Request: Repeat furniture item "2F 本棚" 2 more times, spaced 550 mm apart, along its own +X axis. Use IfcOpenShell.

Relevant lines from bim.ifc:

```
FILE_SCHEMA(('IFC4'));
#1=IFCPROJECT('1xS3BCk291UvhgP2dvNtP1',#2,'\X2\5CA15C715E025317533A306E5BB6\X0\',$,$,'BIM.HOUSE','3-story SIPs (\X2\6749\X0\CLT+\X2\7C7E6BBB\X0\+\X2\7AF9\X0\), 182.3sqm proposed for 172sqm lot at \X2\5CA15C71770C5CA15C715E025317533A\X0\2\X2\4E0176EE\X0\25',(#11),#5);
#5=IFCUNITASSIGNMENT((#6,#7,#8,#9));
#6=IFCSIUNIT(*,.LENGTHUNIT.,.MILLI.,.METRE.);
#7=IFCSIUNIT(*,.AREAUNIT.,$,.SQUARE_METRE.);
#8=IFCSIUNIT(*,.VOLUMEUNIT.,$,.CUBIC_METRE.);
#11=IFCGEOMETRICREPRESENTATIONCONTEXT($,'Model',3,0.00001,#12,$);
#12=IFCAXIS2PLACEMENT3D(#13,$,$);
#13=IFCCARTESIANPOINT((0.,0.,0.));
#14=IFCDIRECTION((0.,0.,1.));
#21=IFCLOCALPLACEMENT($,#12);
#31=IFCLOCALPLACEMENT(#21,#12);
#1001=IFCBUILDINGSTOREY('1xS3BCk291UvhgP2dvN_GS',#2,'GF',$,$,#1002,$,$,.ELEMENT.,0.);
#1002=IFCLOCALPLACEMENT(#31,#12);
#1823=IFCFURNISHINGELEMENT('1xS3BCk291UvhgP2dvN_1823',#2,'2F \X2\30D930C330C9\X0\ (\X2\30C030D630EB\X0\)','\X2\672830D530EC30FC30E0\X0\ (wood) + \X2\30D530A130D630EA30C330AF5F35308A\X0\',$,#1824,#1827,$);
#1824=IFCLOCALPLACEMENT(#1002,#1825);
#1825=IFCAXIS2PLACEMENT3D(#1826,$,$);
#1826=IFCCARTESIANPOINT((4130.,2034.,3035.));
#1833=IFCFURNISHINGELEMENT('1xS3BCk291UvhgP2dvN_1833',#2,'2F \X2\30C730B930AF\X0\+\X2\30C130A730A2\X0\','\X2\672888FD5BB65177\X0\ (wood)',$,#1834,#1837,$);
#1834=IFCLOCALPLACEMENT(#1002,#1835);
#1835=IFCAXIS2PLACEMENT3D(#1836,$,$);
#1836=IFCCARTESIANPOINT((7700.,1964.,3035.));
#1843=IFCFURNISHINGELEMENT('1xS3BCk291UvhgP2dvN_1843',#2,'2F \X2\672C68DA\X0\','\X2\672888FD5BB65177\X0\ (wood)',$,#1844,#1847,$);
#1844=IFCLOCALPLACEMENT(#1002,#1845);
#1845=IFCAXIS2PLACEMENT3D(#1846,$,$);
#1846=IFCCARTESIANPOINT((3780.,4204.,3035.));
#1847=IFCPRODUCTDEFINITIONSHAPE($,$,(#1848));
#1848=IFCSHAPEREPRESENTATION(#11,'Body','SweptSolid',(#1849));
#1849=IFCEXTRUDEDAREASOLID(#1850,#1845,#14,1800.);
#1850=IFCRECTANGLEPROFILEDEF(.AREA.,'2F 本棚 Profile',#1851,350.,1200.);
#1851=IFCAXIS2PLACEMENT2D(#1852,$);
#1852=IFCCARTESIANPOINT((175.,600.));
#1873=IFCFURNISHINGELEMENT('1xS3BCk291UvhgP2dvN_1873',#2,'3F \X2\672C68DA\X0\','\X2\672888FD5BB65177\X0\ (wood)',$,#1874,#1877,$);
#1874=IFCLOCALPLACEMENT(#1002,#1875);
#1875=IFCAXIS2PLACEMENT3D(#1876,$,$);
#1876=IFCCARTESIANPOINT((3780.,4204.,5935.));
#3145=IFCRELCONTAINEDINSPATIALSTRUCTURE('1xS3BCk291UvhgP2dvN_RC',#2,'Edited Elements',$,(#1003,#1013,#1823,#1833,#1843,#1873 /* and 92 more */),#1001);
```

```python
import ifcopenshell
import ifcopenshell.api.geometry
import ifcopenshell.api.root
import ifcopenshell.util.element
import ifcopenshell.util.placement
import ifcopenshell.util.unit

model = ifcopenshell.open("bim.ifc")
unit_scale = ifcopenshell.util.unit.calculate_unit_scale(model)


def reuse_history(source, copy):
    """copy_class also copies each property set's owner history, people and application; keep the originals."""
    for rel in copy.IsDefinedBy:
        if rel.is_a("IfcRelDefinesByProperties") and (history := rel.RelatingPropertyDefinition.OwnerHistory):
            rel.RelatingPropertyDefinition.OwnerHistory = source.OwnerHistory
            ifcopenshell.util.element.remove_deep2(model, history)


source = model.by_id(1843)
base = ifcopenshell.util.placement.get_local_placement(source.ObjectPlacement)
step = base[:3, 0] * 0.55 / unit_scale

for i in range(1, 3):
    copy = ifcopenshell.api.root.copy_class(model, product=source)
    copy.Representation = ifcopenshell.util.element.copy_deep(
        model, source.Representation, exclude=["IfcGeometricRepresentationContext", "IfcRepresentationMap"]
    )
    reuse_history(source, copy)
    matrix = base.copy()
    matrix[:3, 3] += i * step
    print("added at", matrix[:3, 3].round(3) + 0.0)
    ifcopenshell.api.geometry.edit_object_placement(model, product=copy, matrix=matrix, is_si=False)

model.write("bim_updated.ifc")
```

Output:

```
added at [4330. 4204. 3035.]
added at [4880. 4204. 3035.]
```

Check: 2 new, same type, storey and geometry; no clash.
